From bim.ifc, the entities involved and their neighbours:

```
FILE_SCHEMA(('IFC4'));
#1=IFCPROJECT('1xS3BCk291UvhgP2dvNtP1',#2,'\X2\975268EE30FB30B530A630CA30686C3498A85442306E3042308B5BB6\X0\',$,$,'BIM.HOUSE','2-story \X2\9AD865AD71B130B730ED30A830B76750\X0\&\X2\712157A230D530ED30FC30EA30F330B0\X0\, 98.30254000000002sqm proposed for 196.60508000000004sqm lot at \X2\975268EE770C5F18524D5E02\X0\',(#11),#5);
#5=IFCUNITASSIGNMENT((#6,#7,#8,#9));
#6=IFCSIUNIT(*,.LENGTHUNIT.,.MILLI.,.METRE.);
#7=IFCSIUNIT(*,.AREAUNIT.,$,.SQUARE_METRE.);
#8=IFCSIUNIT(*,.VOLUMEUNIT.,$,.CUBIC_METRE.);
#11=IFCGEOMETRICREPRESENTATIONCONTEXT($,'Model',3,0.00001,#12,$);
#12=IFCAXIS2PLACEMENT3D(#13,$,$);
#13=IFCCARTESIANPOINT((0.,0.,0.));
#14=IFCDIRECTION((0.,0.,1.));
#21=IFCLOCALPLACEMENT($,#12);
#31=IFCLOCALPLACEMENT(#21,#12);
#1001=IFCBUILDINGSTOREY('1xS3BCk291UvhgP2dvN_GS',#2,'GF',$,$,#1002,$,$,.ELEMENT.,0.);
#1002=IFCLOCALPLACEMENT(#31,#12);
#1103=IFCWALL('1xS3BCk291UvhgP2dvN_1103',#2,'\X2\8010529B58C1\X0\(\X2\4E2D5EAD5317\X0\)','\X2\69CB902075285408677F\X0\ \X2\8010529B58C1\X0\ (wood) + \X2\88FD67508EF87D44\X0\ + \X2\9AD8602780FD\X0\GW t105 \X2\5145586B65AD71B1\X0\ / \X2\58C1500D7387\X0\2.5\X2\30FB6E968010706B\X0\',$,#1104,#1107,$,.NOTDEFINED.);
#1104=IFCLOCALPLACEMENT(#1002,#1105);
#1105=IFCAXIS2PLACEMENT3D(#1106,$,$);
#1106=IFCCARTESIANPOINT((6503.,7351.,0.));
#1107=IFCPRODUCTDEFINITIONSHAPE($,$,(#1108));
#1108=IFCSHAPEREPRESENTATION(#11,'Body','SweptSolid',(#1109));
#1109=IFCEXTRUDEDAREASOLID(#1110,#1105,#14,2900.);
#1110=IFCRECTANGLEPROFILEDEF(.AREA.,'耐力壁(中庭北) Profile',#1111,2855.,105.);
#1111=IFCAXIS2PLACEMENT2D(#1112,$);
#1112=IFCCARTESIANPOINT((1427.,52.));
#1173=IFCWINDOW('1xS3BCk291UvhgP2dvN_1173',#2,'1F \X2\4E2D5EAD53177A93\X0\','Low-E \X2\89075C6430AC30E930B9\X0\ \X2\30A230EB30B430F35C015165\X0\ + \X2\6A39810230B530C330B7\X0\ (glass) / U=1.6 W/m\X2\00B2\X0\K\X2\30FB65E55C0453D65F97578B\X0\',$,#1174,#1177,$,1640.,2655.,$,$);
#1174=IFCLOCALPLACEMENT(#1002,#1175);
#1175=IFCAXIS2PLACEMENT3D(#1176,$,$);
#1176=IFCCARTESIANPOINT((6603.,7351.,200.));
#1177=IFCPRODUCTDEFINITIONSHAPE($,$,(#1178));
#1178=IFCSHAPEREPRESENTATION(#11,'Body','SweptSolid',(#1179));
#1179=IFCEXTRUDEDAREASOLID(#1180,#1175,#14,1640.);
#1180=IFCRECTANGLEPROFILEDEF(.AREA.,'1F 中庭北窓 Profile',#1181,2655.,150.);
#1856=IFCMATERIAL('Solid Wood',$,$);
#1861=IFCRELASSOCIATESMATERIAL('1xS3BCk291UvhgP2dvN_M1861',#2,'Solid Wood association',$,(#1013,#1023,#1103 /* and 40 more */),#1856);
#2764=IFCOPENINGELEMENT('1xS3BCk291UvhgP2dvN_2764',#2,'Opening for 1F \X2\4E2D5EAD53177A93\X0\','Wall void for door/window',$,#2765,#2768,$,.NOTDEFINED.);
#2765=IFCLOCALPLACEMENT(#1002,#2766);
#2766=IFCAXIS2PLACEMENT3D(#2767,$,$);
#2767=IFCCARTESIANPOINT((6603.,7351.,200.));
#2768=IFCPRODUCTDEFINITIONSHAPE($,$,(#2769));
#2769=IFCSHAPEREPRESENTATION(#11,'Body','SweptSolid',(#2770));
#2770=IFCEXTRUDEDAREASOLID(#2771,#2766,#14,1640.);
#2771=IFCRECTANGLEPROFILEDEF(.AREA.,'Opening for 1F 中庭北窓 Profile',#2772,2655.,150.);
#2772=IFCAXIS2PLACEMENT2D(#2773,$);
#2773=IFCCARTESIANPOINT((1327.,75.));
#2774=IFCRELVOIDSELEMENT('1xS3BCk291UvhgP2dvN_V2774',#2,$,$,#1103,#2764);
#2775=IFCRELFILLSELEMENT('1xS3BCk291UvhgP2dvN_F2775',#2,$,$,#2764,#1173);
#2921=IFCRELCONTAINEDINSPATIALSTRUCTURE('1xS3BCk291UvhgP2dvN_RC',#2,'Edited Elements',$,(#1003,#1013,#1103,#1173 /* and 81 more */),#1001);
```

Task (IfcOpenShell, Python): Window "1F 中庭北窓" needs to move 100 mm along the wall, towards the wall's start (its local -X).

```python
import ifcopenshell
import ifcopenshell.api.geometry
import ifcopenshell.util.placement
import ifcopenshell.util.unit

model = ifcopenshell.open("bim.ifc")
unit_scale = ifcopenshell.util.unit.calculate_unit_scale(model)

window = model.by_guid("1xS3BCk291UvhgP2dvN_1173")
opening = window.FillsVoids[0].RelatingOpeningElement
wall = opening.VoidsElements[0].RelatingBuildingElement

wall_matrix = ifcopenshell.util.placement.get_local_placement(wall.ObjectPlacement)
shift = wall_matrix[:3, 0] * -0.1 / unit_scale
before = ifcopenshell.util.placement.get_local_placement(window.ObjectPlacement)[:3, 3].copy()

# The window is not placed relative to its opening, so move both.
for product in (opening, window):
    matrix = ifcopenshell.util.placement.get_local_placement(product.ObjectPlacement)
    matrix[:3, 3] += shift
    ifcopenshell.api.geometry.edit_object_placement(model, product=product, matrix=matrix, is_si=False)

after = ifcopenshell.util.placement.get_local_placement(window.ObjectPlacement)[:3, 3]
print("window moved by", (after - before).round(3) + 0.0)

model.write("bim-out.ifc")
```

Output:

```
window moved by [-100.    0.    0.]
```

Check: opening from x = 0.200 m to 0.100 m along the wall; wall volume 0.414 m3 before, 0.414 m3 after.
